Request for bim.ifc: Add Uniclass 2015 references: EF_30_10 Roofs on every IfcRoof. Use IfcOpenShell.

First a look at what the model holds.

```python
import ifcopenshell

model = ifcopenshell.open("bim.ifc")
print(model.schema)
print("classifications:", [c.Name for c in model.by_type("IfcClassification")])
for ifc_class in ("IfcDoor", "IfcRoof", "IfcStair", "IfcWall", "IfcWindow"):
    print(ifc_class, len(model.by_type(ifc_class)))
```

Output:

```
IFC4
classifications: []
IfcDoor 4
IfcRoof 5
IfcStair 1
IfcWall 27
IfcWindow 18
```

```python
import ifcopenshell
import ifcopenshell.api.classification

model = ifcopenshell.open("bim.ifc")

system = ifcopenshell.api.classification.add_classification(model, classification="Uniclass 2015")

codes = {
    "IfcRoof": ("EF_30_10", "Roofs"),
}
for ifc_class, (code, name) in codes.items():
    products = model.by_type(ifc_class)
    ifcopenshell.api.classification.add_reference(
        model, products=products, classification=system, identification=code, name=name
    )
    print(code, len(products))

model.write("bim_edited.ifc")
```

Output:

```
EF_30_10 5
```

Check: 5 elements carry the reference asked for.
